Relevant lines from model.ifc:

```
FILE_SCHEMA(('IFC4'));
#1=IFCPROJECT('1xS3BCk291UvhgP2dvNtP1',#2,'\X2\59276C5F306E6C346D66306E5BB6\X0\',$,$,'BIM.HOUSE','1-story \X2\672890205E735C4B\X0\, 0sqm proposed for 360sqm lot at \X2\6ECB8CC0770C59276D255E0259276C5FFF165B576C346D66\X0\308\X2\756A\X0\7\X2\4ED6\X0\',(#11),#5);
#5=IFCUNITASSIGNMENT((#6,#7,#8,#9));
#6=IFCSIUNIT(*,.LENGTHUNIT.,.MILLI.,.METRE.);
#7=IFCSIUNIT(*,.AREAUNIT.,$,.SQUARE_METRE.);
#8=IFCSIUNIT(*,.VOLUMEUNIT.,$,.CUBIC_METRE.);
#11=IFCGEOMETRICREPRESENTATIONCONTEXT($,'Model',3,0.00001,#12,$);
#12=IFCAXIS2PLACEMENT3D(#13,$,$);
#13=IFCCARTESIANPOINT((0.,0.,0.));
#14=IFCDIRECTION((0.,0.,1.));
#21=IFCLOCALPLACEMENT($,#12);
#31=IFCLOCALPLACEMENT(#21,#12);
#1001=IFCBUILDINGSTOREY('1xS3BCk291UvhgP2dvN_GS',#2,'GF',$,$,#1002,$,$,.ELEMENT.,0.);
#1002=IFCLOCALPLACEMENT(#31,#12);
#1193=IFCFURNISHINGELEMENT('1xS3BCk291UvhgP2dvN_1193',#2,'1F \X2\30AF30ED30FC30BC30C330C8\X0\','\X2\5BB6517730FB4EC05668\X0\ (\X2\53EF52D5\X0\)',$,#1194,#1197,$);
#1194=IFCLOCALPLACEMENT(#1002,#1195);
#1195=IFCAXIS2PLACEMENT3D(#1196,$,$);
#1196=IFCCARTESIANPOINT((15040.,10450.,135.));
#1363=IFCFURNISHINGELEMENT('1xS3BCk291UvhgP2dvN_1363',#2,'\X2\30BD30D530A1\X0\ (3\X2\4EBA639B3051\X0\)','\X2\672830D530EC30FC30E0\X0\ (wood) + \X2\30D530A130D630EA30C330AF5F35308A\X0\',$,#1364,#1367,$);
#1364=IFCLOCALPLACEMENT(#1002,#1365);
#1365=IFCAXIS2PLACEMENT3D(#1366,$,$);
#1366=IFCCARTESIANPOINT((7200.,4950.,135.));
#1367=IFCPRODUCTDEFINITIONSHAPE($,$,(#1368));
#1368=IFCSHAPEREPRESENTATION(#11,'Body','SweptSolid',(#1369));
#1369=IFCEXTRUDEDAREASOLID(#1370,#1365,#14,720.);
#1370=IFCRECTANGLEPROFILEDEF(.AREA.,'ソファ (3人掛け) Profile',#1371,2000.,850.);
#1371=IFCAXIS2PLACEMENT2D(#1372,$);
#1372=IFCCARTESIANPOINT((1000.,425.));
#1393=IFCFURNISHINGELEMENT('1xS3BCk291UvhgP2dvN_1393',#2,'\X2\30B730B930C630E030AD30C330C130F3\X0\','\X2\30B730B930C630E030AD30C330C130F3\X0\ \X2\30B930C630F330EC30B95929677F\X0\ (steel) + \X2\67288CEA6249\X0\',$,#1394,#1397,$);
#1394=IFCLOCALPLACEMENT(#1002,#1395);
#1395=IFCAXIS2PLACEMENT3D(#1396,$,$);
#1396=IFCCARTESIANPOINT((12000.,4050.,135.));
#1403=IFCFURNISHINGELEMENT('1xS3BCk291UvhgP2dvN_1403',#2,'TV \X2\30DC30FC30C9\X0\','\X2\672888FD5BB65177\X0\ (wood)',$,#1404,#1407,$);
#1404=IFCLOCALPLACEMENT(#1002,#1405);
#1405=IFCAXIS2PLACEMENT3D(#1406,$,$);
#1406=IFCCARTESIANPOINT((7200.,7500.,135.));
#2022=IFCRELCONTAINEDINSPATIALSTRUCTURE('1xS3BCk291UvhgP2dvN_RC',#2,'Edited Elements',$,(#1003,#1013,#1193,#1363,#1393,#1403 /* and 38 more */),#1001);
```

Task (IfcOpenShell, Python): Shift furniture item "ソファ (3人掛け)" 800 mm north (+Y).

```python
import ifcopenshell
import ifcopenshell.api.geometry
import ifcopenshell.util.placement
import ifcopenshell.util.unit

model = ifcopenshell.open("model.ifc")
unit_scale = ifcopenshell.util.unit.calculate_unit_scale(model)

item = model.by_guid("1xS3BCk291UvhgP2dvN_1363")
matrix = ifcopenshell.util.placement.get_local_placement(item.ObjectPlacement)
matrix[1, 3] += 0.8 / unit_scale
ifcopenshell.api.geometry.edit_object_placement(model, product=item, matrix=matrix, is_si=False)

print(ifcopenshell.util.placement.get_local_placement(item.ObjectPlacement).round(3) + 0.0)

model.write("model_updated.ifc")
```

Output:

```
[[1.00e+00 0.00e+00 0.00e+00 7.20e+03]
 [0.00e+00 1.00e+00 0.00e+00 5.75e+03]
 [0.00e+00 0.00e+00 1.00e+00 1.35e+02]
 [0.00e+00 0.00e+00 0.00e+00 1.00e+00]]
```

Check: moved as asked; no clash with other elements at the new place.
